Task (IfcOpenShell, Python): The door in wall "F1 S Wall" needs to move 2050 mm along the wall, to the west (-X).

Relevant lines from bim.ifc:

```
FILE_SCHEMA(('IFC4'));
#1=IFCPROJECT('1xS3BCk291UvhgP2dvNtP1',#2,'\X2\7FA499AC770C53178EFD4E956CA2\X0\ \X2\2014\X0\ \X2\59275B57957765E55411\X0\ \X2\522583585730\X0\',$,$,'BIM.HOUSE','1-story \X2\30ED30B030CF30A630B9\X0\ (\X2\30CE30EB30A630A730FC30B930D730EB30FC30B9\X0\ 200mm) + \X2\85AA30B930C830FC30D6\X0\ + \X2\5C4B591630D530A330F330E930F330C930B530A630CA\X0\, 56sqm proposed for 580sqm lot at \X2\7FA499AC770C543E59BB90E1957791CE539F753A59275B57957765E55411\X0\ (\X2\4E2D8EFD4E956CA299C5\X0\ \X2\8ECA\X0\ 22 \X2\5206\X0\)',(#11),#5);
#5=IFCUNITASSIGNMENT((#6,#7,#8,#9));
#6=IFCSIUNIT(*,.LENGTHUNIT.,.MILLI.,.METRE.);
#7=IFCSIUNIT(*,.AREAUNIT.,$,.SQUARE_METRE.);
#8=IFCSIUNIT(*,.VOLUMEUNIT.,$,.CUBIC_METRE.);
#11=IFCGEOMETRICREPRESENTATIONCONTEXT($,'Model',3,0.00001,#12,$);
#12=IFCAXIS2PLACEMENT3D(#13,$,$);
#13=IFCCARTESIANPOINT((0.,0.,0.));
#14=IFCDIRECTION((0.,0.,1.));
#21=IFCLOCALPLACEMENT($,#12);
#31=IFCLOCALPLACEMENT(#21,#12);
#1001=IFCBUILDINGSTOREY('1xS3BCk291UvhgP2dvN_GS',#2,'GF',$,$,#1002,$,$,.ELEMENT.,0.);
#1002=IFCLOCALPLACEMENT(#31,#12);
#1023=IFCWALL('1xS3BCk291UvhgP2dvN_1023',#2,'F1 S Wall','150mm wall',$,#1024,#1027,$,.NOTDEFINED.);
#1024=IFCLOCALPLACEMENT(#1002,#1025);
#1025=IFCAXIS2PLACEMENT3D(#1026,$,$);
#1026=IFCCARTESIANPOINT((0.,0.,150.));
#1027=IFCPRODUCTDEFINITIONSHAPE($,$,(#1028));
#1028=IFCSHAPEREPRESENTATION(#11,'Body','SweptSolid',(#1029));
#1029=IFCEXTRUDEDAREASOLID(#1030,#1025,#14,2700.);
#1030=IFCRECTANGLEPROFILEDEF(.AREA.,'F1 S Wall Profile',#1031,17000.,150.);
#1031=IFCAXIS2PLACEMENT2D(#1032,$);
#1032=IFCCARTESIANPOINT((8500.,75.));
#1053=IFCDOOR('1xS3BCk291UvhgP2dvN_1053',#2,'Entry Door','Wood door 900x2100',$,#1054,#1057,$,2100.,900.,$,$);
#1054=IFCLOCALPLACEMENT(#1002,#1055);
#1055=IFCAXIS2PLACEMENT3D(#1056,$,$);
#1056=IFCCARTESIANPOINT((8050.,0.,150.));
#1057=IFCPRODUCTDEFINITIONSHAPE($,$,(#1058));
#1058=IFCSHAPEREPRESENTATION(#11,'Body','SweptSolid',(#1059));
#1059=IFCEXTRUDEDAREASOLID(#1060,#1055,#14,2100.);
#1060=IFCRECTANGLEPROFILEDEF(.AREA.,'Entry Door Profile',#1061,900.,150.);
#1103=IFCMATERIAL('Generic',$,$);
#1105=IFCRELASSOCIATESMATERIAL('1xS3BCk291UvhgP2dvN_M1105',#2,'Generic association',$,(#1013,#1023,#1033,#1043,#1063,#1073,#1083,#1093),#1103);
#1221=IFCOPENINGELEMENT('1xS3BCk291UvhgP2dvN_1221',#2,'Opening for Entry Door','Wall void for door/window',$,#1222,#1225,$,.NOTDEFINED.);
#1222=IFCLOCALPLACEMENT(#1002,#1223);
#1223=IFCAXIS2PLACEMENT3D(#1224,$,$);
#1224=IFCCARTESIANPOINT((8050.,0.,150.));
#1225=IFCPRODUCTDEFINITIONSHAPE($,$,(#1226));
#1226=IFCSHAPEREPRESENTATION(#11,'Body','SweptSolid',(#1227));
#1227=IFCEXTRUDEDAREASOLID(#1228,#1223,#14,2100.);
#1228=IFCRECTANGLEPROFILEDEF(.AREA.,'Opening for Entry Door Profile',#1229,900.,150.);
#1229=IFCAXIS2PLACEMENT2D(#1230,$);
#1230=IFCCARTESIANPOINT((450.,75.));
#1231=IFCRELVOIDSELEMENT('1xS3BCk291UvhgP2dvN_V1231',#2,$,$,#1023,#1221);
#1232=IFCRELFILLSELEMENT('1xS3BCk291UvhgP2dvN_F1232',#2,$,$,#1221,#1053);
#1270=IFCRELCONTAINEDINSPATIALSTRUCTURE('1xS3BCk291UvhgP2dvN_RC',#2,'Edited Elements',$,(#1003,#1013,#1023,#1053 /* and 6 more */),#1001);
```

```python
import ifcopenshell
import ifcopenshell.api.geometry
import ifcopenshell.util.placement
import ifcopenshell.util.unit

model = ifcopenshell.open("bim.ifc")
unit_scale = ifcopenshell.util.unit.calculate_unit_scale(model)

door = model.by_guid("1xS3BCk291UvhgP2dvN_1053")
opening = door.FillsVoids[0].RelatingOpeningElement
wall = opening.VoidsElements[0].RelatingBuildingElement

wall_matrix = ifcopenshell.util.placement.get_local_placement(wall.ObjectPlacement)
shift = wall_matrix[:3, 0] * -2.05 / unit_scale
before = ifcopenshell.util.placement.get_local_placement(door.ObjectPlacement)[:3, 3].copy()

# The door is not placed relative to its opening, so move both.
for product in (opening, door):
    matrix = ifcopenshell.util.placement.get_local_placement(product.ObjectPlacement)
    matrix[:3, 3] += shift
    ifcopenshell.api.geometry.edit_object_placement(model, product=product, matrix=matrix, is_si=False)

after = ifcopenshell.util.placement.get_local_placement(door.ObjectPlacement)[:3, 3]
print("door moved by", (after - before).round(3) + 0.0)

model.write("bim_edited.ifc")
```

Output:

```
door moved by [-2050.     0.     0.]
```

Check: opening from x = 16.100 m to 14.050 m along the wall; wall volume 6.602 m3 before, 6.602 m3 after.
